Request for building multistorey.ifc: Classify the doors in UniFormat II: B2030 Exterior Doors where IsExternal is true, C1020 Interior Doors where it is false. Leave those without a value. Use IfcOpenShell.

First a look at what the model holds.

```python
import ifcopenshell
import ifcopenshell.util.element

model = ifcopenshell.open("building multistorey.ifc")
print(model.schema)
print("classifications:", [c.Name for c in model.by_type("IfcClassification")])
values = [ifcopenshell.util.element.get_pset(e, "Pset_DoorCommon", "IsExternal") for e in model.by_type("IfcDoor")]
for value in (True, False, None):
    print("IsExternal", value, values.count(value))
```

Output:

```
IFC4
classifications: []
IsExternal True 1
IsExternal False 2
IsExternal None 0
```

```python
import ifcopenshell
import ifcopenshell.api.classification
import ifcopenshell.util.element

model = ifcopenshell.open("building multistorey.ifc")

system = ifcopenshell.api.classification.add_classification(model, classification="UniFormat II")

doors = model.by_type("IfcDoor")
external = {e: ifcopenshell.util.element.get_pset(e, "Pset_DoorCommon", "IsExternal") for e in doors}
for flag, code, name in ((True, "B2030", "Exterior Doors"), (False, "C1020", "Interior Doors")):
    products = [e for e in doors if external[e] is flag]
    ifcopenshell.api.classification.add_reference(
        model, products=products, classification=system, identification=code, name=name
    )
    print(code, len(products))

model.write("building multistorey_edited.ifc")
```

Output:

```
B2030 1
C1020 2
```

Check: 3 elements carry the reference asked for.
